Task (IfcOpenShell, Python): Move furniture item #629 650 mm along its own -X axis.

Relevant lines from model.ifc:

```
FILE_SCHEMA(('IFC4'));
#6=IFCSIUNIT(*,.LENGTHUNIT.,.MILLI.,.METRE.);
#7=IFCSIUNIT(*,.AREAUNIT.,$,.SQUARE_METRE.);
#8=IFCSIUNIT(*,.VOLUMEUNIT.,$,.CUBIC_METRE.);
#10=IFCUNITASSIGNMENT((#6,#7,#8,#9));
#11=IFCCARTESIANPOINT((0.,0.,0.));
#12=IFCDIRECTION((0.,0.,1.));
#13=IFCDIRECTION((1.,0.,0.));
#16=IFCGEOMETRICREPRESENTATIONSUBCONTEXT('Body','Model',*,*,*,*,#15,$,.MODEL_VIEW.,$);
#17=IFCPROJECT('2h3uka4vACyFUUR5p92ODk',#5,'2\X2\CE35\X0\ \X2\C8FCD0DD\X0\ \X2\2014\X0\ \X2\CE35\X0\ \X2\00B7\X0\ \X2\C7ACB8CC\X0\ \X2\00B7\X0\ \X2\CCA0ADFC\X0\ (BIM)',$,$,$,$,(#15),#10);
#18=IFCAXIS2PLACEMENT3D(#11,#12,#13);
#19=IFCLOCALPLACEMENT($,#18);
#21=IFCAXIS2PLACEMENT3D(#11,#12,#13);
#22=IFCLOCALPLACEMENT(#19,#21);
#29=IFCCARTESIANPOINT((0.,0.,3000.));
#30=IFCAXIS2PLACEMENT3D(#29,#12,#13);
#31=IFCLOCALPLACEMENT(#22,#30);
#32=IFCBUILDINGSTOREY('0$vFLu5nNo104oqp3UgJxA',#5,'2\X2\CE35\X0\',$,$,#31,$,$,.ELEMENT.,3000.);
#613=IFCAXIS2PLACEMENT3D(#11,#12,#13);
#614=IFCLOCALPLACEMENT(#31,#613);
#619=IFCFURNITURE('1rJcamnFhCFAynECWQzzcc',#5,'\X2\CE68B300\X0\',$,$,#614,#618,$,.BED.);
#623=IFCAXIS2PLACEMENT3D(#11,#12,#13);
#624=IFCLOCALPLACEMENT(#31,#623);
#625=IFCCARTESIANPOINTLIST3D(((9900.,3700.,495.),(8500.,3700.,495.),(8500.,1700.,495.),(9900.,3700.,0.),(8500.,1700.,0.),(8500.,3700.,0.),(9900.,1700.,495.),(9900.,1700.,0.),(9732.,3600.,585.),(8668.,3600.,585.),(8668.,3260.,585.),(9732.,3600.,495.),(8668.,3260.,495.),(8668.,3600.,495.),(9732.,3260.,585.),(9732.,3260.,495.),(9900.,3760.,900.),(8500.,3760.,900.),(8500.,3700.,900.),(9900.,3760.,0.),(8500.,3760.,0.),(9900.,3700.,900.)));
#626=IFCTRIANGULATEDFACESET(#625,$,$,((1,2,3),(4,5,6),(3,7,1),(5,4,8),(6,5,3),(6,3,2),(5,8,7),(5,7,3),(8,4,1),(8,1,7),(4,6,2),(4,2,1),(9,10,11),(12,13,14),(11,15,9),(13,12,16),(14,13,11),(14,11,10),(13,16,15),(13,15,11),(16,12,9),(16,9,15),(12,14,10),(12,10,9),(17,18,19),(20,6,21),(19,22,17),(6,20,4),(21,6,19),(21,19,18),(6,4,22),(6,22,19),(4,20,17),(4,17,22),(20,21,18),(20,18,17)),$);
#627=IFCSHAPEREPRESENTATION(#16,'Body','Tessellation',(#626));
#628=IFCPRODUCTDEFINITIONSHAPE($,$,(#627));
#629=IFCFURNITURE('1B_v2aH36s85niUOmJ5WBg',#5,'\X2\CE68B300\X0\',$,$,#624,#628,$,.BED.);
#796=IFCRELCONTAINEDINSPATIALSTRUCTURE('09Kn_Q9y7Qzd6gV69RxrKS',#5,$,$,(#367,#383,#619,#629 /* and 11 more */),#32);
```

```python
import ifcopenshell
import ifcopenshell.api.geometry
import ifcopenshell.util.placement

model = ifcopenshell.open("model.ifc")

item = model.by_guid("1B_v2aH36s85niUOmJ5WBg")
matrix = ifcopenshell.util.placement.get_local_placement(item.ObjectPlacement)
matrix[:3, 3] -= matrix[:3, 0] * 650.0
ifcopenshell.api.geometry.edit_object_placement(model, product=item, matrix=matrix, is_si=False)

print(ifcopenshell.util.placement.get_local_placement(item.ObjectPlacement).round(3) + 0.0)

model.write("model_rev.ifc")
```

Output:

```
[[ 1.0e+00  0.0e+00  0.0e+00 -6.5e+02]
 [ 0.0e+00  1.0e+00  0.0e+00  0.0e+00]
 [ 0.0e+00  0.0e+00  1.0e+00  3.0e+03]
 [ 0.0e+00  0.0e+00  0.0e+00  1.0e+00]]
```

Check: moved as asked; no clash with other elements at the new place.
